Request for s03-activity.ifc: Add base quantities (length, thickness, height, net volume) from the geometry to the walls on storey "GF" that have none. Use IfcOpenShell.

First a look at what the model holds.

```python
import ifcopenshell
import ifcopenshell.util.element
import ifcopenshell.util.unit

model = ifcopenshell.open("s03-activity.ifc")
print(model.schema)
for unit_type in ("LENGTHUNIT", "AREAUNIT", "VOLUMEUNIT"):
    print(unit_type, ifcopenshell.util.unit.calculate_unit_scale(model, unit_type))
storey = next(s for s in model.by_type("IfcBuildingStorey") if s.Name == "GF")
walls = [e for e in ifcopenshell.util.element.get_decomposition(storey) if e.is_a("IfcWall")]
for e in sorted(walls, key=lambda e: e.id()):
    print(e.id(), e.is_a(), e.Name, list(ifcopenshell.util.element.get_psets(e, qtos_only=True)), sep=" | ")
```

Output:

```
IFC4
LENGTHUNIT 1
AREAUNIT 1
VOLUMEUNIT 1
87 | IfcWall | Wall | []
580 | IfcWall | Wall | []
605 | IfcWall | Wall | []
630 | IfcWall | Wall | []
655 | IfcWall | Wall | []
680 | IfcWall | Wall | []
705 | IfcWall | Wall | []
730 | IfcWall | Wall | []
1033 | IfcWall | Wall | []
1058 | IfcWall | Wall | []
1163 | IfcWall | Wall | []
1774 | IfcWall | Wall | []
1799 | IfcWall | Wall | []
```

```python
import ifcopenshell
import ifcopenshell.api.pset
import ifcopenshell.geom
import ifcopenshell.util.element
import ifcopenshell.util.shape
import ifcopenshell.util.unit

model = ifcopenshell.open("s03-activity.ifc")
unit_scale = ifcopenshell.util.unit.calculate_unit_scale(model)
volume_scale = ifcopenshell.util.unit.calculate_unit_scale(model, "VOLUMEUNIT")
settings = ifcopenshell.geom.settings()

storey = next(s for s in model.by_type("IfcBuildingStorey") if s.Name == "GF")
walls = [e for e in ifcopenshell.util.element.get_decomposition(storey) if e.is_a("IfcWall")]

for e in sorted(walls, key=lambda e: e.id()):
    if ifcopenshell.util.element.get_psets(e, qtos_only=True, should_inherit=False):
        continue
    # Geometry comes back in metres, in the element's own axes.
    shape = ifcopenshell.geom.create_shape(settings, e)
    values = {
        "Length": ifcopenshell.util.shape.get_x(shape.geometry) / unit_scale,
        "Width": ifcopenshell.util.shape.get_y(shape.geometry) / unit_scale,
        "Height": ifcopenshell.util.shape.get_z(shape.geometry) / unit_scale,
        "NetVolume": ifcopenshell.util.shape.get_volume(shape.geometry) / volume_scale,
    }
    qto = ifcopenshell.api.pset.add_qto(model, product=e, name="Qto_WallBaseQuantities")
    ifcopenshell.api.pset.edit_qto(model, qto=qto, properties=values)
    print(e.id(), {k: round(v, 3) for k, v in values.items()})

model.write("s03-activity_updated.ifc")
```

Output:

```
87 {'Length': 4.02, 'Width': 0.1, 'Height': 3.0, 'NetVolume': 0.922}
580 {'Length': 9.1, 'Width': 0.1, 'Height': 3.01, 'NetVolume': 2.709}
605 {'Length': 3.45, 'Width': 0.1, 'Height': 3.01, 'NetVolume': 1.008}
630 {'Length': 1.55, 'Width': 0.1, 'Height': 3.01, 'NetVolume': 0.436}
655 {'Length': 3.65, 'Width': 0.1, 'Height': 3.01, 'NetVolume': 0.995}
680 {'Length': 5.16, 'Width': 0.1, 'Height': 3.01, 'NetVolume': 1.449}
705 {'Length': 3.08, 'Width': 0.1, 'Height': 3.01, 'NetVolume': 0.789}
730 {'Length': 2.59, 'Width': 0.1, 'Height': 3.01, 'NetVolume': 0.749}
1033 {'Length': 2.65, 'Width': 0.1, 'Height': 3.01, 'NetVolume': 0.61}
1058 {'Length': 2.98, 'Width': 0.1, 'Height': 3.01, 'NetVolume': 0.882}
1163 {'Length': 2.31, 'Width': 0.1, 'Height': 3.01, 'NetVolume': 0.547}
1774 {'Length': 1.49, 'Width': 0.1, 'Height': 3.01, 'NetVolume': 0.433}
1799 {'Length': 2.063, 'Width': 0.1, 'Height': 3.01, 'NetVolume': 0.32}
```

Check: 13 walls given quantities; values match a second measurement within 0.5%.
